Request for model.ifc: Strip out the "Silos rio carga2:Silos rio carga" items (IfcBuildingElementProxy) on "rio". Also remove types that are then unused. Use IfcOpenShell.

First a look at what the model holds.

```python
import ifcopenshell
import ifcopenshell.util.element

model = ifcopenshell.open("model.ifc")
print(model.schema)
storey = next(s for s in model.by_type("IfcBuildingStorey") if s.Name == "rio")
proxies = [e for e in ifcopenshell.util.element.get_decomposition(storey) if e.is_a("IfcBuildingElementProxy")]
seen = {}
for e in proxies:
    element_type = ifcopenshell.util.element.get_type(e)
    name = element_type.Name if element_type not in (None, e) else None
    seen[name] = seen.get(name, 0) + 1
for name, count in sorted(seen.items(), key=str):
    print(count, "x", name)
```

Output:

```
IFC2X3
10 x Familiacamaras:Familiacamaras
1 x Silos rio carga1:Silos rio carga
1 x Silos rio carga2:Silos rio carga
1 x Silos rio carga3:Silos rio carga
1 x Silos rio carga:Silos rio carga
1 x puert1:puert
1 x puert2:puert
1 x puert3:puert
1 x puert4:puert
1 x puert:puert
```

```python
import ifcopenshell
import ifcopenshell.api.root
import ifcopenshell.util.element

model = ifcopenshell.open("model.ifc")

storey = next(s for s in model.by_type("IfcBuildingStorey") if s.Name == "rio")
proxies = [e for e in ifcopenshell.util.element.get_decomposition(storey) if e.is_a("IfcBuildingElementProxy")]
targets = [e for e in proxies if (t := ifcopenshell.util.element.get_type(e)) not in (None, e) and t.Name == "Silos rio carga2:Silos rio carga"]
types = {ifcopenshell.util.element.get_type(e) for e in targets} - {None, *targets}

for e in targets:
    ifcopenshell.api.root.remove_product(model, product=e)
print(len(targets), "removed")

unused = [t for t in types if not ifcopenshell.util.element.get_types(t)]
for t in unused:
    ifcopenshell.api.root.remove_product(model, product=t)
print(len(unused), "unused types removed")

model.write("model_rev.ifc")
```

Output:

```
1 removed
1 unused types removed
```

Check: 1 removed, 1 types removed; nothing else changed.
